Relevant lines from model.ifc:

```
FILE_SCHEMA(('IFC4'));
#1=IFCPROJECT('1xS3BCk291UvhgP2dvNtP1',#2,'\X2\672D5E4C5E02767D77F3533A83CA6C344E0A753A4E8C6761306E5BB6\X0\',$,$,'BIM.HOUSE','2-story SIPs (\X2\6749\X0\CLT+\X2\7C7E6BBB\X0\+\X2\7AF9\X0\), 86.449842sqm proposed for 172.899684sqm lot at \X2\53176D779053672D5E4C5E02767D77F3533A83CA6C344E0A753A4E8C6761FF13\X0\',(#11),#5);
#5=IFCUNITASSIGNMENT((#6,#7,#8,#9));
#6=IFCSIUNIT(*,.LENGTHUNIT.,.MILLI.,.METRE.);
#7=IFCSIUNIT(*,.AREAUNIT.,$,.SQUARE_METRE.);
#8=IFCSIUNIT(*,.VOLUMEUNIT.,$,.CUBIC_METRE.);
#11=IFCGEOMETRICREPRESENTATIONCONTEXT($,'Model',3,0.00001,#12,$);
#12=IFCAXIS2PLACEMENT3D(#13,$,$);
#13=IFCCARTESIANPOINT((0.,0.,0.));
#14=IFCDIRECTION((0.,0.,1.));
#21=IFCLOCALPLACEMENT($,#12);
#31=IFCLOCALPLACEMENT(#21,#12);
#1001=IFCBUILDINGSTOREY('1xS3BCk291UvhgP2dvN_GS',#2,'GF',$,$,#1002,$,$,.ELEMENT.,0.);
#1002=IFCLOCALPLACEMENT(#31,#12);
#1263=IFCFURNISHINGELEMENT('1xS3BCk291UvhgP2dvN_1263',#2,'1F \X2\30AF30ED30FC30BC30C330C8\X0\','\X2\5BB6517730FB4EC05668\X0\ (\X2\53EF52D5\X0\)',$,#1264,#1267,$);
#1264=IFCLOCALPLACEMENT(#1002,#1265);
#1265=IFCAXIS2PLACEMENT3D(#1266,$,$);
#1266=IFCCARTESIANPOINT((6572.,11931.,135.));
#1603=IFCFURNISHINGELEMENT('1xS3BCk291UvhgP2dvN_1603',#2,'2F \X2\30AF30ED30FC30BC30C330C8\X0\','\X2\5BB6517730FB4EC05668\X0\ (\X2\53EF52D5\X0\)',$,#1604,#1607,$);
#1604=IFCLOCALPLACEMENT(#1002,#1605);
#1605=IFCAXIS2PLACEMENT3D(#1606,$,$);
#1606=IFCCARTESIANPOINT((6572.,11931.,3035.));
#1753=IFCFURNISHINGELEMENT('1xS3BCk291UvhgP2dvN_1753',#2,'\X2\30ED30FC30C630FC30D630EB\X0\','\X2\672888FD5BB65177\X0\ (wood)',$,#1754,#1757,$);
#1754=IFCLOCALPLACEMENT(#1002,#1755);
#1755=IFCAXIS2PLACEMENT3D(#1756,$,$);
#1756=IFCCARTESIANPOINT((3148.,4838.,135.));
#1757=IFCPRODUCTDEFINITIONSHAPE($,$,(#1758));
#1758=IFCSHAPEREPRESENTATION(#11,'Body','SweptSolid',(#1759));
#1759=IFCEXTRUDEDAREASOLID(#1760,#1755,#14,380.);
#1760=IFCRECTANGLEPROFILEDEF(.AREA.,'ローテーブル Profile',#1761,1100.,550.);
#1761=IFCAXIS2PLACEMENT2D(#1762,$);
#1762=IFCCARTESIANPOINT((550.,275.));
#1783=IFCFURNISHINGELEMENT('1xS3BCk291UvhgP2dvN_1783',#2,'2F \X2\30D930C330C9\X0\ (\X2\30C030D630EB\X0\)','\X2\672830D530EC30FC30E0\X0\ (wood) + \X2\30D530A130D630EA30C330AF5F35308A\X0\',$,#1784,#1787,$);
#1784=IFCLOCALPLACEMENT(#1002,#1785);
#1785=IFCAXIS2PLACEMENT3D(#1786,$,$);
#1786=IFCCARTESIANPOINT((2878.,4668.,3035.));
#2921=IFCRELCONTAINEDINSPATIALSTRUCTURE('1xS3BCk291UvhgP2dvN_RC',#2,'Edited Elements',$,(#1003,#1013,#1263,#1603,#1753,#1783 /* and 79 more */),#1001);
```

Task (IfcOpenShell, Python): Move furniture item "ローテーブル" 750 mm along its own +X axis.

```python
import ifcopenshell
import ifcopenshell.api.geometry
import ifcopenshell.util.placement

model = ifcopenshell.open("model.ifc")

item = model.by_guid("1xS3BCk291UvhgP2dvN_1753")
matrix = ifcopenshell.util.placement.get_local_placement(item.ObjectPlacement)
matrix[:3, 3] += matrix[:3, 0] * 750.0
ifcopenshell.api.geometry.edit_object_placement(model, product=item, matrix=matrix, is_si=False)

print(ifcopenshell.util.placement.get_local_placement(item.ObjectPlacement).round(3) + 0.0)

model.write("model-out.ifc")
```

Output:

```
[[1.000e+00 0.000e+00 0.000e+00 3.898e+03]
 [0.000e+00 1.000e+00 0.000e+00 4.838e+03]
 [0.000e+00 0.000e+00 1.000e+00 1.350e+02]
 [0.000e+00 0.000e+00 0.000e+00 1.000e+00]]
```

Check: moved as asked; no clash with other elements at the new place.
